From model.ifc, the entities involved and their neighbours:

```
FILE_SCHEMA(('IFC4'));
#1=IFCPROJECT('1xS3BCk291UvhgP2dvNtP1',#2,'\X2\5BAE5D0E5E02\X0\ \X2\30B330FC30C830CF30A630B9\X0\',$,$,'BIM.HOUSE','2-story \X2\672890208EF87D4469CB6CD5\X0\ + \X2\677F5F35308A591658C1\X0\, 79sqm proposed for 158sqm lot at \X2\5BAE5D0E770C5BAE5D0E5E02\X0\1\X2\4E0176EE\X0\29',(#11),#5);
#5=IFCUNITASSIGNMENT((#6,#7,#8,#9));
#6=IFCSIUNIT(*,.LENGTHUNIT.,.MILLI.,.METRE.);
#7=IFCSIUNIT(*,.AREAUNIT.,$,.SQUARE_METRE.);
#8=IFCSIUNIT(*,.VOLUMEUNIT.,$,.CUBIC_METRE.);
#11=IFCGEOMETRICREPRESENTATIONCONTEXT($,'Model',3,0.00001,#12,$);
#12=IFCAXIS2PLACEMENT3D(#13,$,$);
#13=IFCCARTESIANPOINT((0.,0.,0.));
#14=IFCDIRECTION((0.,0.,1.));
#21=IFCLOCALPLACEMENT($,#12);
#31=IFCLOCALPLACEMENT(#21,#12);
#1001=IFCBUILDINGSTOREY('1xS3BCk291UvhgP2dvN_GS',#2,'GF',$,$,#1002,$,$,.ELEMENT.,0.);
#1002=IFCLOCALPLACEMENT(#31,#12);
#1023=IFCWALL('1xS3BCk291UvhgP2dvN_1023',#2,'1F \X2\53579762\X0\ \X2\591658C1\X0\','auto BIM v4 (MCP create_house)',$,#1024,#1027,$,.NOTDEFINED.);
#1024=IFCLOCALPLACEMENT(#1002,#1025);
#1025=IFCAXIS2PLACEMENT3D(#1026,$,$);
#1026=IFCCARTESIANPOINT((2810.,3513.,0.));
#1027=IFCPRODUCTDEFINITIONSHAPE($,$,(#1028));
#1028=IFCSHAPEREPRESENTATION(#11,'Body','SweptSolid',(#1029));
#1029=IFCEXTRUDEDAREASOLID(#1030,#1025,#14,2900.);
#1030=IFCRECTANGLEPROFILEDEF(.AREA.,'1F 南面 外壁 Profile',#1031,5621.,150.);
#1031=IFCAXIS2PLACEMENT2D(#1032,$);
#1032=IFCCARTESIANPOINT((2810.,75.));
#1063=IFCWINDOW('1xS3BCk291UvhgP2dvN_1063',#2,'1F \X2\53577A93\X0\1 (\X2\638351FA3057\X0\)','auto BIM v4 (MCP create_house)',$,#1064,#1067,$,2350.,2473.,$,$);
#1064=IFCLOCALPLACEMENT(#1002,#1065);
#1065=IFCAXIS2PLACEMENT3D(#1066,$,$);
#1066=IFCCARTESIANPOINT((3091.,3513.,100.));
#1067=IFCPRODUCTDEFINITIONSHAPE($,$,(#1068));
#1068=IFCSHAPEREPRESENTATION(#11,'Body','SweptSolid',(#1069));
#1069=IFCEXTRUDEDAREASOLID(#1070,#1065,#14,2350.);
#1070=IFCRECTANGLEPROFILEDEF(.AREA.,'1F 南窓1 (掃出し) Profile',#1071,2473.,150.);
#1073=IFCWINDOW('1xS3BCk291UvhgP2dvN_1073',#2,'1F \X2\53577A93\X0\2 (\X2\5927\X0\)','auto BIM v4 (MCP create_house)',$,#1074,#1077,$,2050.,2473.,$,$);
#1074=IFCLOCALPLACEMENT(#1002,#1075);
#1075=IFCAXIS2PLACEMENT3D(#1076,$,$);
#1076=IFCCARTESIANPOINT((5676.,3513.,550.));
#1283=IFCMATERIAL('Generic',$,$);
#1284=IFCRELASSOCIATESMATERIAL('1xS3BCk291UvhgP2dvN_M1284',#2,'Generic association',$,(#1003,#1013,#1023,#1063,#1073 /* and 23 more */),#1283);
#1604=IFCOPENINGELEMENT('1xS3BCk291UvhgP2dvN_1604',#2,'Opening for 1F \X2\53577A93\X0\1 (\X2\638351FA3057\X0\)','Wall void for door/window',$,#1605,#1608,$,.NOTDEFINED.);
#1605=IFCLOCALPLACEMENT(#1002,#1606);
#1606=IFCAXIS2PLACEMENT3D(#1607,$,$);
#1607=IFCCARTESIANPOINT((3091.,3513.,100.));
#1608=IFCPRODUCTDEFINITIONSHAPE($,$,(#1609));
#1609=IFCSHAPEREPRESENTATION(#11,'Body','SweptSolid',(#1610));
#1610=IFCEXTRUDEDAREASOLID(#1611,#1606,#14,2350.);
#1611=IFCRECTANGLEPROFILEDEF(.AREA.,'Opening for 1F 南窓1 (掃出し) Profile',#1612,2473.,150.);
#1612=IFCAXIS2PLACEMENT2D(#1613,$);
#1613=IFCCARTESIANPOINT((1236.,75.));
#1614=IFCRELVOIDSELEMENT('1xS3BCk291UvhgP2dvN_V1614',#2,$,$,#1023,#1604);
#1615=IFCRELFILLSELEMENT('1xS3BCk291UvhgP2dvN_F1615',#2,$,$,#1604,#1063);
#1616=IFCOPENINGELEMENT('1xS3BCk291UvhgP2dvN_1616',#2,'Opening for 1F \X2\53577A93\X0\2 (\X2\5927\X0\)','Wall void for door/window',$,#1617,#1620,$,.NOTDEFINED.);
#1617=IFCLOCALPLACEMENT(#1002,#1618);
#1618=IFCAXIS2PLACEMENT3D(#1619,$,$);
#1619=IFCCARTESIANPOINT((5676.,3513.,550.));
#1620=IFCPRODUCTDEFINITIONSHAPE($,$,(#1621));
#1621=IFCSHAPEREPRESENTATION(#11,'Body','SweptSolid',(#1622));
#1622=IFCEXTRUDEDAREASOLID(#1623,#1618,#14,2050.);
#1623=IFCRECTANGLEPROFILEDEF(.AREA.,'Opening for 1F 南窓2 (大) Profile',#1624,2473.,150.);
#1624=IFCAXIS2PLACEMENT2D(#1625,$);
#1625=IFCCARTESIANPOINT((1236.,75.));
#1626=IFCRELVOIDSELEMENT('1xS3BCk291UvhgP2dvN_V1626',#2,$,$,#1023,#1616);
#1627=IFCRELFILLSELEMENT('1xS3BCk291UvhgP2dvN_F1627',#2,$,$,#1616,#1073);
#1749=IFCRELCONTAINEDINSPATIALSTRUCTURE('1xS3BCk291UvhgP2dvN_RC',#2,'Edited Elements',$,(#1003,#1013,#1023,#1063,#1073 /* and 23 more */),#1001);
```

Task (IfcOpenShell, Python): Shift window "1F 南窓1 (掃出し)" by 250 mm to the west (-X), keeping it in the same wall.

```python
import ifcopenshell
import ifcopenshell.api.geometry
import ifcopenshell.util.placement

model = ifcopenshell.open("model.ifc")

window = model.by_guid("1xS3BCk291UvhgP2dvN_1063")
opening = window.FillsVoids[0].RelatingOpeningElement
wall = opening.VoidsElements[0].RelatingBuildingElement

wall_matrix = ifcopenshell.util.placement.get_local_placement(wall.ObjectPlacement)
shift = wall_matrix[:3, 0] * -250.0
before = ifcopenshell.util.placement.get_local_placement(window.ObjectPlacement)[:3, 3].copy()

# The window is not placed relative to its opening, so move both.
for product in (opening, window):
    matrix = ifcopenshell.util.placement.get_local_placement(product.ObjectPlacement)
    matrix[:3, 3] += shift
    ifcopenshell.api.geometry.edit_object_placement(model, product=product, matrix=matrix, is_si=False)

after = ifcopenshell.util.placement.get_local_placement(window.ObjectPlacement)[:3, 3]
print("window moved by", (after - before).round(3) + 0.0)

model.write("model-out.ifc")
```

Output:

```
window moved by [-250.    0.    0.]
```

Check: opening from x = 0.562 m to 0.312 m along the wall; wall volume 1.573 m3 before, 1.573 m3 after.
